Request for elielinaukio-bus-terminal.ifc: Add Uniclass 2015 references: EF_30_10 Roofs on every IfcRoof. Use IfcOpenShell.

First a look at what the model holds.

```python
import ifcopenshell

model = ifcopenshell.open("elielinaukio-bus-terminal.ifc")
print(model.schema)
print("classifications:", [c.Name for c in model.by_type("IfcClassification")])
for ifc_class in ("IfcDoor", "IfcRoof", "IfcStair", "IfcWall", "IfcWindow"):
    print(ifc_class, len(model.by_type(ifc_class)))
```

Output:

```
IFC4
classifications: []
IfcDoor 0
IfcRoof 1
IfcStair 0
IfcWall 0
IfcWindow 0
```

```python
import ifcopenshell
import ifcopenshell.api.classification

model = ifcopenshell.open("elielinaukio-bus-terminal.ifc")

system = ifcopenshell.api.classification.add_classification(model, classification="Uniclass 2015")

codes = {
    "IfcRoof": ("EF_30_10", "Roofs"),
}
for ifc_class, (code, name) in codes.items():
    products = model.by_type(ifc_class)
    ifcopenshell.api.classification.add_reference(
        model, products=products, classification=system, identification=code, name=name
    )
    print(code, len(products))

model.write("elielinaukio-bus-terminal_updated.ifc")
```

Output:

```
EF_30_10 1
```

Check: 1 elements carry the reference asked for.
